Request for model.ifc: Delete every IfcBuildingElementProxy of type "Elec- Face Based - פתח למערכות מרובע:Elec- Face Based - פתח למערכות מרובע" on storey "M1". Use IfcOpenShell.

First a look at what the model holds.

```python
import ifcopenshell
import ifcopenshell.util.element

model = ifcopenshell.open("model.ifc")
print(model.schema)
storey = next(s for s in model.by_type("IfcBuildingStorey") if s.Name == "M1")
proxies = [e for e in ifcopenshell.util.element.get_decomposition(storey) if e.is_a("IfcBuildingElementProxy")]
seen = {}
for e in proxies:
    element_type = ifcopenshell.util.element.get_type(e)
    name = element_type.Name if element_type not in (None, e) else None
    seen[name] = seen.get(name, 0) + 1
for name, count in sorted(seen.items(), key=str):
    print(count, "x", name)
```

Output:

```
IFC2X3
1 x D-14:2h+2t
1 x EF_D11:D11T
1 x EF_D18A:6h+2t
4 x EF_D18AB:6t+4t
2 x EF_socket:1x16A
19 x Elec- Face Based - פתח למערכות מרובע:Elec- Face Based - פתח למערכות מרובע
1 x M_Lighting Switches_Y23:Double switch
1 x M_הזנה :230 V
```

```python
import ifcopenshell
import ifcopenshell.api.root
import ifcopenshell.util.element

model = ifcopenshell.open("model.ifc")

storey = next(s for s in model.by_type("IfcBuildingStorey") if s.Name == "M1")
proxies = [e for e in ifcopenshell.util.element.get_decomposition(storey) if e.is_a("IfcBuildingElementProxy")]
targets = [e for e in proxies if (t := ifcopenshell.util.element.get_type(e)) not in (None, e) and t.Name == "Elec- Face Based - פתח למערכות מרובע:Elec- Face Based - פתח למערכות מרובע"]

for e in targets:
    ifcopenshell.api.root.remove_product(model, product=e)
print(len(targets), "removed")

model.write("model_edited.ifc")
```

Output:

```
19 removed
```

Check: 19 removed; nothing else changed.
